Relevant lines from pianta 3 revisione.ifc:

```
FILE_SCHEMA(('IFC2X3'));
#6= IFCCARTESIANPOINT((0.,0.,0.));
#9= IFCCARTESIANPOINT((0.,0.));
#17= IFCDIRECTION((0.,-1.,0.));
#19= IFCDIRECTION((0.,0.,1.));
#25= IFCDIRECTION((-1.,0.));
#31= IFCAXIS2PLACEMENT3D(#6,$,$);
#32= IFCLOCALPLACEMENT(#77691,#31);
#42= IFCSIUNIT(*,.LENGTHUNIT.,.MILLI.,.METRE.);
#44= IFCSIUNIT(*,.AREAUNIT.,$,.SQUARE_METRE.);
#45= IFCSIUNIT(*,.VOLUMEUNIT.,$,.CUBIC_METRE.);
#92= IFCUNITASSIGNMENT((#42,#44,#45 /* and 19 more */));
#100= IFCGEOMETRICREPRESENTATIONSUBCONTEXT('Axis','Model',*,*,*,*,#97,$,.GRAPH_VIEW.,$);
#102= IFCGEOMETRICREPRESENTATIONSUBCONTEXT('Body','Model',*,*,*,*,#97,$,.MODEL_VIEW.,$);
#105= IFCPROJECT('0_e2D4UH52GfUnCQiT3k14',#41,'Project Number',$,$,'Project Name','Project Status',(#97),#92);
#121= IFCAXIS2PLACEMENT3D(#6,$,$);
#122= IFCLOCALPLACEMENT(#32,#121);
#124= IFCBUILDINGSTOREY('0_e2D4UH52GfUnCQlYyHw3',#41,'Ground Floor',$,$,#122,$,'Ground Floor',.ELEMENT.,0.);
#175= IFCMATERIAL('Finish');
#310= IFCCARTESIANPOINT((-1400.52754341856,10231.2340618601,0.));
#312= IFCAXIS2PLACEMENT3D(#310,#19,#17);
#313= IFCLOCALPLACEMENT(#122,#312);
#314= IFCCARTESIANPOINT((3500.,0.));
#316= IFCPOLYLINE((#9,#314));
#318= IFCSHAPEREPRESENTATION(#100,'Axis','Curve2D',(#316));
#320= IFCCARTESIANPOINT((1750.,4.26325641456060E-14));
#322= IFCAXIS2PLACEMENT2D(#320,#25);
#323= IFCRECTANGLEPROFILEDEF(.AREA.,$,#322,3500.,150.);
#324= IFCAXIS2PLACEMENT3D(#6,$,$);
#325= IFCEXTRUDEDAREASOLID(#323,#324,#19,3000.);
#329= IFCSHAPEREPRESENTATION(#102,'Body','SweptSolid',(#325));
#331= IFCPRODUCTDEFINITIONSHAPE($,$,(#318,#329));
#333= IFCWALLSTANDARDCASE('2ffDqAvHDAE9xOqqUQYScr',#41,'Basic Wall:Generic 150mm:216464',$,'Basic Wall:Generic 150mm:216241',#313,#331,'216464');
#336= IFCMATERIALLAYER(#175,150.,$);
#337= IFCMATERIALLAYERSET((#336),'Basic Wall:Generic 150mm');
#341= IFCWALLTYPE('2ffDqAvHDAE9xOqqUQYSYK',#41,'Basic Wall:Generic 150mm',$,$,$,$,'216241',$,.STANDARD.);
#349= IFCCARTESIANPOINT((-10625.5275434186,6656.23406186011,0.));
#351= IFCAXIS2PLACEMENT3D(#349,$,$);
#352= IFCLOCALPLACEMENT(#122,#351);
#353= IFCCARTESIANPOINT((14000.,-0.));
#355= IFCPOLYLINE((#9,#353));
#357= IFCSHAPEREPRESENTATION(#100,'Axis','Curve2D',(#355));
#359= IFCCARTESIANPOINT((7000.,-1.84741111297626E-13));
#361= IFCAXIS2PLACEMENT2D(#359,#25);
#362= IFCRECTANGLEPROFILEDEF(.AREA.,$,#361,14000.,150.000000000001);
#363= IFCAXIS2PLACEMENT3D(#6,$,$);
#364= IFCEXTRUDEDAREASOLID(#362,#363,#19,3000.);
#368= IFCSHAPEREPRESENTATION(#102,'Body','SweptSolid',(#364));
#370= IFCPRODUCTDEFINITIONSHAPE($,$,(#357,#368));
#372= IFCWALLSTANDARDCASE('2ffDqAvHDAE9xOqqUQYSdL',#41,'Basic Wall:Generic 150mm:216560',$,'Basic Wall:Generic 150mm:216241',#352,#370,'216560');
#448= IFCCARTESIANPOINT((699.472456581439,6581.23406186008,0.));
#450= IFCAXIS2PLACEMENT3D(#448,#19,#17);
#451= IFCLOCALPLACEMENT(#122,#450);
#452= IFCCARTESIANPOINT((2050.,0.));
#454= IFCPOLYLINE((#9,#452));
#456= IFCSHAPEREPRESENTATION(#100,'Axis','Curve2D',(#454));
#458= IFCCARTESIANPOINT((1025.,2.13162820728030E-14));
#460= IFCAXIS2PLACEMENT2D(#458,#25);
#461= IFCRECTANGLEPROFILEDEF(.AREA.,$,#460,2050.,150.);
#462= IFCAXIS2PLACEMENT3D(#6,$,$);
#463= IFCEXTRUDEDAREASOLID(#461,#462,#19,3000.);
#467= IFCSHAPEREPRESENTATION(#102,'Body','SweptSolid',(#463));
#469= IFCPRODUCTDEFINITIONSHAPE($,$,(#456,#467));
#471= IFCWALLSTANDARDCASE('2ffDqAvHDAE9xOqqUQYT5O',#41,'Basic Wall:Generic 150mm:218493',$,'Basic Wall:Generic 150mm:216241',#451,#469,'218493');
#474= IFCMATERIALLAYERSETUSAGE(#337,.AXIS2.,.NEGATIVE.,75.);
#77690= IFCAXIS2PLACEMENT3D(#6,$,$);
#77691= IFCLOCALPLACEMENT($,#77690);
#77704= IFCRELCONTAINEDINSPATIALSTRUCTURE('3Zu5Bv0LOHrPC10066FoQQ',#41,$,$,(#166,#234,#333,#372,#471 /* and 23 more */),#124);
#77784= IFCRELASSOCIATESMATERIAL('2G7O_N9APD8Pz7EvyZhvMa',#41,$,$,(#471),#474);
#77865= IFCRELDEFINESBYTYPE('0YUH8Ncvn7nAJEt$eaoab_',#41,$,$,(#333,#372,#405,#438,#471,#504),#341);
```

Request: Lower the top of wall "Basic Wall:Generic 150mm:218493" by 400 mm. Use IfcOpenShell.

```python
import ifcopenshell
import ifcopenshell.geom
import ifcopenshell.util.representation
import ifcopenshell.util.shape
import ifcopenshell.util.unit

model = ifcopenshell.open("pianta 3 revisione.ifc")
unit_scale = ifcopenshell.util.unit.calculate_unit_scale(model)
settings = ifcopenshell.geom.settings()


def volume(element):
    """Net volume in cubic metres, openings subtracted."""
    shape = ifcopenshell.geom.create_shape(settings, element)
    return ifcopenshell.util.shape.get_volume(shape.geometry)


wall = model.by_guid("2ffDqAvHDAE9xOqqUQYT5O")
before = volume(wall)

body = ifcopenshell.util.representation.get_representation(wall, "Model", "Body")
solid = body.Items[0]
old_height = solid.Depth
solid.Depth -= 0.4 / unit_scale
after = volume(wall)

print(f"height {old_height:g} -> {solid.Depth:g}, volume {before:.3f} -> {after:.3f} m3")

model.write("pianta 3 revisione_updated.ifc")
```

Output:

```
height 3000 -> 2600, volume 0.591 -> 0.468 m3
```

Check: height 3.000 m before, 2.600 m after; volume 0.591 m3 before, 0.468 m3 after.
